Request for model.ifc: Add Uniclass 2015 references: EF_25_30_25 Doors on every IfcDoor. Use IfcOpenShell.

First a look at what the model holds.

```python
import ifcopenshell

model = ifcopenshell.open("model.ifc")
print(model.schema)
print("classifications:", [c.Name for c in model.by_type("IfcClassification")])
for ifc_class in ("IfcDoor", "IfcRoof", "IfcStair", "IfcWall", "IfcWindow"):
    print(ifc_class, len(model.by_type(ifc_class)))
```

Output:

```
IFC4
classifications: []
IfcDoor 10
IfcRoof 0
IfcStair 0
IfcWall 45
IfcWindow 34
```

```python
import ifcopenshell
import ifcopenshell.api.classification

model = ifcopenshell.open("model.ifc")

system = ifcopenshell.api.classification.add_classification(model, classification="Uniclass 2015")

codes = {
    "IfcDoor": ("EF_25_30_25", "Doors"),
}
for ifc_class, (code, name) in codes.items():
    products = model.by_type(ifc_class)
    ifcopenshell.api.classification.add_reference(
        model, products=products, classification=system, identification=code, name=name
    )
    print(code, len(products))

model.write("model_rev.ifc")
```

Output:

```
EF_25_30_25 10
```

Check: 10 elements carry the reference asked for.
